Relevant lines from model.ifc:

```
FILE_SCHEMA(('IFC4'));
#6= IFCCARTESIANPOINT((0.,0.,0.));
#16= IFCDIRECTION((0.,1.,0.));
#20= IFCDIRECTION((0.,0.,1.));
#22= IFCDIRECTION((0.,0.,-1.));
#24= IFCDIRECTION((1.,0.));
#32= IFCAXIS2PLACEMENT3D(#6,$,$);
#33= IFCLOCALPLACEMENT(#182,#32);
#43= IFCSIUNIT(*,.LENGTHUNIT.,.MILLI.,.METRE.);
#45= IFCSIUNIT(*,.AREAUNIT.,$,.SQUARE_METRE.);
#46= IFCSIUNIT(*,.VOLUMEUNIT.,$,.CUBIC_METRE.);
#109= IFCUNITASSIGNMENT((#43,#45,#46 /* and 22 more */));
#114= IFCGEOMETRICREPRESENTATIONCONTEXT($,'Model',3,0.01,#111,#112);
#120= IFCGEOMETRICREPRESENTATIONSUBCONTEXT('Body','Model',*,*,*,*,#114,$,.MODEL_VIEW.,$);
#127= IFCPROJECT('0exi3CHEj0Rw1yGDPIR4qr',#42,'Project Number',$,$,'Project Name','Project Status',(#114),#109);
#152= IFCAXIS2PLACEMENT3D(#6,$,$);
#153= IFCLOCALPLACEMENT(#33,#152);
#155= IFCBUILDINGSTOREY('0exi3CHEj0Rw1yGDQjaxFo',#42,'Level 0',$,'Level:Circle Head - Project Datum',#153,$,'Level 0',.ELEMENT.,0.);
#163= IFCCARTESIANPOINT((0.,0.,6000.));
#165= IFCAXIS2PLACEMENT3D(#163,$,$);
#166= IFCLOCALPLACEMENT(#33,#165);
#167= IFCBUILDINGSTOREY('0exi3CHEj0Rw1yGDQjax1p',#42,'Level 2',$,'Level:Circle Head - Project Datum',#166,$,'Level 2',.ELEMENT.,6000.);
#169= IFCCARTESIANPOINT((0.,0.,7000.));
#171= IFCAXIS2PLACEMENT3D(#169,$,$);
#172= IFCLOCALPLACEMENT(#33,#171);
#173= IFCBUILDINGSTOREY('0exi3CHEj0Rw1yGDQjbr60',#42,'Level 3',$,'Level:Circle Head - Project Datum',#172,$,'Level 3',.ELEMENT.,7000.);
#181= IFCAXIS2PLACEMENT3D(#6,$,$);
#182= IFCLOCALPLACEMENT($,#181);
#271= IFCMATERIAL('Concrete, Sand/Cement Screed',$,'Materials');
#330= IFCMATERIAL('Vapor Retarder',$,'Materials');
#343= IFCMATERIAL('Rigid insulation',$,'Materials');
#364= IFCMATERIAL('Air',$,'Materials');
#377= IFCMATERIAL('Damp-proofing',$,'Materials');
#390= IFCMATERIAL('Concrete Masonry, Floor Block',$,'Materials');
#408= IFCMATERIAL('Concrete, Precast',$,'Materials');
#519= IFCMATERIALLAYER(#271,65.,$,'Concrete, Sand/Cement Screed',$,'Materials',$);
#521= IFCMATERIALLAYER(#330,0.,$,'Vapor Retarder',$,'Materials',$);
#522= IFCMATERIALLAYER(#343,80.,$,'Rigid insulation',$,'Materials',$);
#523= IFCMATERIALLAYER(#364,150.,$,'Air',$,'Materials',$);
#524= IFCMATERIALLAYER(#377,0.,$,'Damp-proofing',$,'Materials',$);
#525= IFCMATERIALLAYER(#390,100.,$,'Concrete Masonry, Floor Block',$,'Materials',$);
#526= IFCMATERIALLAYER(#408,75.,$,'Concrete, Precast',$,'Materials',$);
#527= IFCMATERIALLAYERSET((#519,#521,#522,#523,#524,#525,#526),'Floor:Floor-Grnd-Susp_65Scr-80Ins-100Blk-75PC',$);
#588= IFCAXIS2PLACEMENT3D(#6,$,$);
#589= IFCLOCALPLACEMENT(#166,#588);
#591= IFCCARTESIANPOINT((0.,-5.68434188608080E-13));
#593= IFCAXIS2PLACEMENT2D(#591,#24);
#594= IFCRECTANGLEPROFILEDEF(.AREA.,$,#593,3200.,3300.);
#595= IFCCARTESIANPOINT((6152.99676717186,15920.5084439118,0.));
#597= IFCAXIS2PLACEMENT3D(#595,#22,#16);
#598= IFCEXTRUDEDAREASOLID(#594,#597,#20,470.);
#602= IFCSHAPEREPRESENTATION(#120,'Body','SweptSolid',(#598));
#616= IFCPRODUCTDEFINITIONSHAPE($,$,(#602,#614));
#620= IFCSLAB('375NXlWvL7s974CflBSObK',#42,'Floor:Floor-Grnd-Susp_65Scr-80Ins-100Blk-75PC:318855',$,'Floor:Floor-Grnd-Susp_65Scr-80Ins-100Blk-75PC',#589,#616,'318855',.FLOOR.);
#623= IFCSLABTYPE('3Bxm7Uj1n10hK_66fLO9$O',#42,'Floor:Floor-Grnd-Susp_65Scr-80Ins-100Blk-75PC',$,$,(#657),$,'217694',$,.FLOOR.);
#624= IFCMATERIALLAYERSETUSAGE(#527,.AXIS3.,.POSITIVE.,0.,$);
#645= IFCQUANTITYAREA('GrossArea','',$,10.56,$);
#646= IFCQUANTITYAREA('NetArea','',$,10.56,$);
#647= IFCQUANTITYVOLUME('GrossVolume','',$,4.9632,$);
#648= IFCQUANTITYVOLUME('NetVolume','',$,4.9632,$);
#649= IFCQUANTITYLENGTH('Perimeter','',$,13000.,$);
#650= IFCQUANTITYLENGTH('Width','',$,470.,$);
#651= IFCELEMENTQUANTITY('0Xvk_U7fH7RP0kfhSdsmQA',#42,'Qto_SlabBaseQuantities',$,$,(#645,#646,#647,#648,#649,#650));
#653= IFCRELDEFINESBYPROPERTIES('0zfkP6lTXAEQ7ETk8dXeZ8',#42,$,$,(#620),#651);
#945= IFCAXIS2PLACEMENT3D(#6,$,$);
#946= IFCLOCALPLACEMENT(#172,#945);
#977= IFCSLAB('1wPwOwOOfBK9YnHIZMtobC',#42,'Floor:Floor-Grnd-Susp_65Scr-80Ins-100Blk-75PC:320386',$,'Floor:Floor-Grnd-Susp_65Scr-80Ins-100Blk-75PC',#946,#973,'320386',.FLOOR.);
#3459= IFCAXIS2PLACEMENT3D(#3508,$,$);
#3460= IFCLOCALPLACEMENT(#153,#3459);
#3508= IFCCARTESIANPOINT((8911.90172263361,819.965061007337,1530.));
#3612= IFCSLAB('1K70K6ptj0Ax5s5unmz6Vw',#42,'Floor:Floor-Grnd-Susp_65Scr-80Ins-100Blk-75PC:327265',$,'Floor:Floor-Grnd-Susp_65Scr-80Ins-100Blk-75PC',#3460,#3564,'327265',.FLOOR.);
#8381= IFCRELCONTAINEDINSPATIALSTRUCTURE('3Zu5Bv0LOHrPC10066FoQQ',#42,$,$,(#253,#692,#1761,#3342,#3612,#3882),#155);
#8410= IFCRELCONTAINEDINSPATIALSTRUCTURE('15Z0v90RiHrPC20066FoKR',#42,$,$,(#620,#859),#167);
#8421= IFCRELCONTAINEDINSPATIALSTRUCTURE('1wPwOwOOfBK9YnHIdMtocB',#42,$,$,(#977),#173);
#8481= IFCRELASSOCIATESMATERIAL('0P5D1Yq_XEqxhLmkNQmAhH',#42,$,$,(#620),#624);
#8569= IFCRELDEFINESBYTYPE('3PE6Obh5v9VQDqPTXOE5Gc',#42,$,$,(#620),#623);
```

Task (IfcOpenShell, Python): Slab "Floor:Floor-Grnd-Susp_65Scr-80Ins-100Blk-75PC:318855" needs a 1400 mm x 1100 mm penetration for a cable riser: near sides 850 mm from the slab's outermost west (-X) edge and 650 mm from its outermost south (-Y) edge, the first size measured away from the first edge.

```python
import numpy as np
import ifcopenshell
import ifcopenshell.api.feature
import ifcopenshell.api.geometry
import ifcopenshell.api.pset
import ifcopenshell.api.root
import ifcopenshell.geom
import ifcopenshell.util.element
import ifcopenshell.util.placement
import ifcopenshell.util.representation
import ifcopenshell.util.shape
import ifcopenshell.util.unit

model = ifcopenshell.open("model.ifc")
unit_scale = ifcopenshell.util.unit.calculate_unit_scale(model)
area_scale = ifcopenshell.util.unit.calculate_unit_scale(model, "AREAUNIT")
volume_scale = ifcopenshell.util.unit.calculate_unit_scale(model, "VOLUMEUNIT")
settings = ifcopenshell.geom.settings()


def volume(element):
    """Net volume in cubic metres, openings subtracted."""
    shape = ifcopenshell.geom.create_shape(settings, element)
    return ifcopenshell.util.shape.get_volume(shape.geometry)


slab = model.by_guid("375NXlWvL7s974CflBSObK")
before = volume(slab)

# Extent in the slab's own axes, in metres. The edges named are its -X and -Y sides.
slab_shape = ifcopenshell.geom.create_shape(settings, slab)
vertices = ifcopenshell.util.shape.get_vertices(slab_shape.geometry)
x_min, y_min, bottom = vertices.min(axis=0)
top = vertices[:, 2].max()

opening = ifcopenshell.api.root.create_entity(model, ifc_class="IfcOpeningElement", name="Cable riser opening", predefined_type="OPENING")
context = ifcopenshell.util.representation.get_context(model, "Model", "Body", "MODEL_VIEW")
width, depth = 1.4, 1.1
outline = [(0.0, 0.0), (width, 0.0), (width, depth), (0.0, depth), (0.0, 0.0)]
# Overshoot both faces by 50 mm so the cut is clean.
shape = ifcopenshell.api.geometry.add_slab_representation(
    model, context=context, depth=top - bottom + 0.1, polyline=outline
)
ifcopenshell.api.geometry.assign_representation(model, product=opening, representation=shape)

matrix = ifcopenshell.util.placement.get_local_placement(slab.ObjectPlacement)
matrix[:, 3] = matrix @ np.append(np.array([x_min + 0.85, y_min + 0.65, bottom - 0.05]) / unit_scale, 1.0)
ifcopenshell.api.geometry.edit_object_placement(model, product=opening, matrix=matrix, is_si=False)
ifcopenshell.api.feature.add_feature(model, feature=opening, element=slab)

after = volume(slab)

# Update the slab's stored quantities.
qto = model.by_id(ifcopenshell.util.element.get_pset(slab, "Qto_SlabBaseQuantities", should_inherit=False)["id"])
ifcopenshell.api.pset.edit_qto(model, qto=qto, properties={
    "NetArea": after / (top - bottom) / area_scale,
    "NetVolume": after / volume_scale,
})

print(f"slab volume {before:.3f} -> {after:.3f} m3")

model.write("model_updated.ifc")
```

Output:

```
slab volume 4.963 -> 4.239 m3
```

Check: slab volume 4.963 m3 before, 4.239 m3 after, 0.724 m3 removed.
